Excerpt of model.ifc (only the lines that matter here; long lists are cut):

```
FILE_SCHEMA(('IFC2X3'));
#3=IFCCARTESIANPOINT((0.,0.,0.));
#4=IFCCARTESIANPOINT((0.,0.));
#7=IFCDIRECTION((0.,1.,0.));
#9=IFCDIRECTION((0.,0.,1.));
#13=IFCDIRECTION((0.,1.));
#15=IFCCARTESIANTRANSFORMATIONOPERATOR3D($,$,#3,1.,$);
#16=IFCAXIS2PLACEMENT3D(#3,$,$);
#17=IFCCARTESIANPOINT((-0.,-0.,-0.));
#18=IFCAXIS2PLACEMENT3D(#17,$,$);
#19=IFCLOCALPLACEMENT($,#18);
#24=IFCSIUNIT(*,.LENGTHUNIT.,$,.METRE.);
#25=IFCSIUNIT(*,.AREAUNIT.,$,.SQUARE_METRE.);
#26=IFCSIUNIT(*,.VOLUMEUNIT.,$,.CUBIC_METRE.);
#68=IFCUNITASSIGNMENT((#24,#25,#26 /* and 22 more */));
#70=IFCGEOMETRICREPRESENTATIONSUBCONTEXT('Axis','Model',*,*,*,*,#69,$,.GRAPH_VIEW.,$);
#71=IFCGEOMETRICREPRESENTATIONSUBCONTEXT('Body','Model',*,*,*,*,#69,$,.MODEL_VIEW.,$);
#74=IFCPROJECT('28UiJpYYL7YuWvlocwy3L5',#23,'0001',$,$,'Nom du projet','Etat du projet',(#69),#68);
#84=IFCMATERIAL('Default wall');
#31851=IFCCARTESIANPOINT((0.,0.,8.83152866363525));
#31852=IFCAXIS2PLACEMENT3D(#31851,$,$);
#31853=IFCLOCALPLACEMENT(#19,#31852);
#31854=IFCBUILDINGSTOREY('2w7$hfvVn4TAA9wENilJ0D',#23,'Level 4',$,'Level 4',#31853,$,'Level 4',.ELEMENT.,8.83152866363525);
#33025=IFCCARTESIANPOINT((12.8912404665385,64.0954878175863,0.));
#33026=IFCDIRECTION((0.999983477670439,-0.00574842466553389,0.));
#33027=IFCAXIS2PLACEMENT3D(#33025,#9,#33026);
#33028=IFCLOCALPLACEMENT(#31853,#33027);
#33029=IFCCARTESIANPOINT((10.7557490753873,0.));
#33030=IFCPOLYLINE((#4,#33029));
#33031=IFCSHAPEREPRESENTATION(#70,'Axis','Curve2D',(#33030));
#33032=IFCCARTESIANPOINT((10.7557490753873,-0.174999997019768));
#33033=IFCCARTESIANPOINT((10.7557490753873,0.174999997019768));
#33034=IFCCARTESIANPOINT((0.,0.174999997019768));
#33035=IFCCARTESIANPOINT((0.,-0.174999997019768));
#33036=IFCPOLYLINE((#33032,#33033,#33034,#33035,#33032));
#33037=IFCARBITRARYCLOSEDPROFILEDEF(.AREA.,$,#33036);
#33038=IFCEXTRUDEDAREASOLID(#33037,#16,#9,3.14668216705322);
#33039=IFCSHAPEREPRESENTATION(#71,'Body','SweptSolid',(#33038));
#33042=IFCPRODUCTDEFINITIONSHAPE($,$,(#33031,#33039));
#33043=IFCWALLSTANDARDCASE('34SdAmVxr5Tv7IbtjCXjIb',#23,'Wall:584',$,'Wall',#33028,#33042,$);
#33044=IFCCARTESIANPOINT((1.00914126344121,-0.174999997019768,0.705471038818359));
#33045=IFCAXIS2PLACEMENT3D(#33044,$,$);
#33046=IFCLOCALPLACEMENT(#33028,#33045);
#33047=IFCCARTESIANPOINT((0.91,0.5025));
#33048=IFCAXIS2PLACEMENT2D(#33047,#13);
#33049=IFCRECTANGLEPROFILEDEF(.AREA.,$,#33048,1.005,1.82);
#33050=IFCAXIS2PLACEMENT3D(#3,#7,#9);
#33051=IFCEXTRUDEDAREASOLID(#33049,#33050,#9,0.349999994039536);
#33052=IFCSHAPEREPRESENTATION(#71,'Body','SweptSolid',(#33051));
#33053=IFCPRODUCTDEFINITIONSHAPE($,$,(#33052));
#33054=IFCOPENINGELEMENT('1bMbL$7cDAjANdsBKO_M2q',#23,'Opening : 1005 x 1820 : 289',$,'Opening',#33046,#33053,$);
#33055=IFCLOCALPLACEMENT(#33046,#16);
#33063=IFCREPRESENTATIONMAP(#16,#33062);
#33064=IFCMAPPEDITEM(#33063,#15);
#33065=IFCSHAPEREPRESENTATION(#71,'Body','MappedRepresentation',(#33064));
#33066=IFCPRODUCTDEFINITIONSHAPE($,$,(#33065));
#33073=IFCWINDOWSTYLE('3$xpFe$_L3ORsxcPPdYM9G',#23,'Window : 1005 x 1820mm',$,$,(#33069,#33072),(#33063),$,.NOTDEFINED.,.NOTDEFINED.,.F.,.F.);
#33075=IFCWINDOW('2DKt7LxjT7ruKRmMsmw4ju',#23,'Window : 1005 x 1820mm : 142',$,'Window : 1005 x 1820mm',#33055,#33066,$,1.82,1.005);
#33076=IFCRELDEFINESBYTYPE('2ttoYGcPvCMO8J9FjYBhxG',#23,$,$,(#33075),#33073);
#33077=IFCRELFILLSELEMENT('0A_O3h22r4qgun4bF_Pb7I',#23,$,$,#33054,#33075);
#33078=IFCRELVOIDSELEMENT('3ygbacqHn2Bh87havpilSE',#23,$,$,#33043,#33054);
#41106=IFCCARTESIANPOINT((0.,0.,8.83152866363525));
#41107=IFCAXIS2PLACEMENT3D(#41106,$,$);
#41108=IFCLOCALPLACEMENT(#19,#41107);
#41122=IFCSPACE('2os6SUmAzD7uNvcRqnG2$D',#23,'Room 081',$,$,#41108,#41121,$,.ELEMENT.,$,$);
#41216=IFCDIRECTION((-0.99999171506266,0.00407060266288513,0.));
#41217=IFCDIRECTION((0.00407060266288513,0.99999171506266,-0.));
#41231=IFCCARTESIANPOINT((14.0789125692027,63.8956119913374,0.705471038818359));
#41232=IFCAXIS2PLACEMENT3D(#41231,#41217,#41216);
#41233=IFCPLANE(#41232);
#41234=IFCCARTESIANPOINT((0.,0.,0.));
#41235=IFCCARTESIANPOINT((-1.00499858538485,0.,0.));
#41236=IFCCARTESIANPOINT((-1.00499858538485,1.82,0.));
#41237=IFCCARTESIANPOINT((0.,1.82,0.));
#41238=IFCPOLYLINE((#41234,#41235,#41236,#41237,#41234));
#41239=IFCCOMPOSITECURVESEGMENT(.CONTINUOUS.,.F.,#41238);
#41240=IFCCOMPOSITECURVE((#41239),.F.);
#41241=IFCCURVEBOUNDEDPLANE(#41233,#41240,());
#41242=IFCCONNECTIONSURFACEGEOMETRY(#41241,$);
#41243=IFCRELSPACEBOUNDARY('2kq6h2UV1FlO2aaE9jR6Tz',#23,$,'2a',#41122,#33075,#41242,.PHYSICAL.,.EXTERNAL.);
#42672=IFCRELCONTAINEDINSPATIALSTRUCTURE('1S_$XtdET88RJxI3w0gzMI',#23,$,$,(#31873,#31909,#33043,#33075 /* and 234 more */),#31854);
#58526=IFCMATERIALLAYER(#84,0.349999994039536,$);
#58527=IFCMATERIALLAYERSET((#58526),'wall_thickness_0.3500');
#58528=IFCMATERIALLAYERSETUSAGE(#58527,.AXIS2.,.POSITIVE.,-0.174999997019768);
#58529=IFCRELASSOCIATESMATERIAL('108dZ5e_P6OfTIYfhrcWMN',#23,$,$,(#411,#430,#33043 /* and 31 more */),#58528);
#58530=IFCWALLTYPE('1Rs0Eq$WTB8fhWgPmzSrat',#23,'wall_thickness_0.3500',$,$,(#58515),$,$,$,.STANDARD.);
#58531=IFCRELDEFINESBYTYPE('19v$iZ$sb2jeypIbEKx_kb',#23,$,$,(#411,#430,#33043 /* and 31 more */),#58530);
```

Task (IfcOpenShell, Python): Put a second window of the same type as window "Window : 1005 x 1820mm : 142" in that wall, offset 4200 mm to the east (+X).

```python
import numpy as np
import ifcopenshell
import ifcopenshell.api.feature
import ifcopenshell.api.geometry
import ifcopenshell.api.root
import ifcopenshell.geom
import ifcopenshell.util.element
import ifcopenshell.util.placement
import ifcopenshell.util.shape
import ifcopenshell.util.unit

model = ifcopenshell.open("model.ifc")
unit_scale = ifcopenshell.util.unit.calculate_unit_scale(model)
settings = ifcopenshell.geom.settings()


def volume(element):
    """Net volume in cubic metres, openings subtracted."""
    shape = ifcopenshell.geom.create_shape(settings, element)
    return ifcopenshell.util.shape.get_volume(shape.geometry)


window = model.by_guid("2DKt7LxjT7ruKRmMsmw4ju")
opening = window.FillsVoids[0].RelatingOpeningElement
wall = opening.VoidsElements[0].RelatingBuildingElement
before = volume(wall)
shift = ifcopenshell.util.placement.get_local_placement(wall.ObjectPlacement)[:3, 0] * 4.2 / unit_scale

# copy_class copies the void relationship, type, container and properties, but no geometry.
new_opening = ifcopenshell.api.root.copy_class(model, product=opening)
new_opening.Representation = ifcopenshell.util.element.copy_deep(
    model, opening.Representation, exclude=["IfcGeometricRepresentationContext", "IfcRepresentationMap"]
)
new_opening.Name = "Opening : 1005 x 1820"
new_window = ifcopenshell.api.root.copy_class(model, product=window)
new_window.Representation = ifcopenshell.util.element.copy_deep(
    model, window.Representation, exclude=["IfcGeometricRepresentationContext", "IfcRepresentationMap"]
)
new_window.Name = "Window : 1005 x 1820mm"
fills = ifcopenshell.api.feature.add_filling(model, opening=new_opening, element=new_window)
fills.OwnerHistory = new_window.OwnerHistory  # required in IFC2X3

for old, new in ((opening, new_opening), (window, new_window)):
    matrix = ifcopenshell.util.placement.get_local_placement(old.ObjectPlacement)
    matrix[:3, 3] += shift
    ifcopenshell.api.geometry.edit_object_placement(model, product=new, matrix=matrix, is_si=False)

# The copied space boundaries still share their surfaces with the original.
for rel in new_window.ProvidesBoundaries:
    if rel.ConnectionGeometry:
        rel.ConnectionGeometry = ifcopenshell.util.element.copy_deep(model, rel.ConnectionGeometry)

# Space boundary surfaces are stored in each space's coordinates; move them too.
for rel in new_window.ProvidesBoundaries:
    if not rel.ConnectionGeometry:
        continue
    surface = rel.ConnectionGeometry.SurfaceOnRelatingElement.BasisSurface
    space_matrix = ifcopenshell.util.placement.get_local_placement(rel.RelatingSpace.ObjectPlacement)
    point = np.array(surface.Position.Location.Coordinates) + space_matrix[:3, :3].T @ shift
    surface.Position = model.createIfcAxis2Placement3D(
        model.createIfcCartesianPoint(point.tolist()), surface.Position.Axis, surface.Position.RefDirection
    )

after = volume(wall)

print(f"wall volume {before:.3f} -> {after:.3f} m3")

model.write("model_v2.ifc")
```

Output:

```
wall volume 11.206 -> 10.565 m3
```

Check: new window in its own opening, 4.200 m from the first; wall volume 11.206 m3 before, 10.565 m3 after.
